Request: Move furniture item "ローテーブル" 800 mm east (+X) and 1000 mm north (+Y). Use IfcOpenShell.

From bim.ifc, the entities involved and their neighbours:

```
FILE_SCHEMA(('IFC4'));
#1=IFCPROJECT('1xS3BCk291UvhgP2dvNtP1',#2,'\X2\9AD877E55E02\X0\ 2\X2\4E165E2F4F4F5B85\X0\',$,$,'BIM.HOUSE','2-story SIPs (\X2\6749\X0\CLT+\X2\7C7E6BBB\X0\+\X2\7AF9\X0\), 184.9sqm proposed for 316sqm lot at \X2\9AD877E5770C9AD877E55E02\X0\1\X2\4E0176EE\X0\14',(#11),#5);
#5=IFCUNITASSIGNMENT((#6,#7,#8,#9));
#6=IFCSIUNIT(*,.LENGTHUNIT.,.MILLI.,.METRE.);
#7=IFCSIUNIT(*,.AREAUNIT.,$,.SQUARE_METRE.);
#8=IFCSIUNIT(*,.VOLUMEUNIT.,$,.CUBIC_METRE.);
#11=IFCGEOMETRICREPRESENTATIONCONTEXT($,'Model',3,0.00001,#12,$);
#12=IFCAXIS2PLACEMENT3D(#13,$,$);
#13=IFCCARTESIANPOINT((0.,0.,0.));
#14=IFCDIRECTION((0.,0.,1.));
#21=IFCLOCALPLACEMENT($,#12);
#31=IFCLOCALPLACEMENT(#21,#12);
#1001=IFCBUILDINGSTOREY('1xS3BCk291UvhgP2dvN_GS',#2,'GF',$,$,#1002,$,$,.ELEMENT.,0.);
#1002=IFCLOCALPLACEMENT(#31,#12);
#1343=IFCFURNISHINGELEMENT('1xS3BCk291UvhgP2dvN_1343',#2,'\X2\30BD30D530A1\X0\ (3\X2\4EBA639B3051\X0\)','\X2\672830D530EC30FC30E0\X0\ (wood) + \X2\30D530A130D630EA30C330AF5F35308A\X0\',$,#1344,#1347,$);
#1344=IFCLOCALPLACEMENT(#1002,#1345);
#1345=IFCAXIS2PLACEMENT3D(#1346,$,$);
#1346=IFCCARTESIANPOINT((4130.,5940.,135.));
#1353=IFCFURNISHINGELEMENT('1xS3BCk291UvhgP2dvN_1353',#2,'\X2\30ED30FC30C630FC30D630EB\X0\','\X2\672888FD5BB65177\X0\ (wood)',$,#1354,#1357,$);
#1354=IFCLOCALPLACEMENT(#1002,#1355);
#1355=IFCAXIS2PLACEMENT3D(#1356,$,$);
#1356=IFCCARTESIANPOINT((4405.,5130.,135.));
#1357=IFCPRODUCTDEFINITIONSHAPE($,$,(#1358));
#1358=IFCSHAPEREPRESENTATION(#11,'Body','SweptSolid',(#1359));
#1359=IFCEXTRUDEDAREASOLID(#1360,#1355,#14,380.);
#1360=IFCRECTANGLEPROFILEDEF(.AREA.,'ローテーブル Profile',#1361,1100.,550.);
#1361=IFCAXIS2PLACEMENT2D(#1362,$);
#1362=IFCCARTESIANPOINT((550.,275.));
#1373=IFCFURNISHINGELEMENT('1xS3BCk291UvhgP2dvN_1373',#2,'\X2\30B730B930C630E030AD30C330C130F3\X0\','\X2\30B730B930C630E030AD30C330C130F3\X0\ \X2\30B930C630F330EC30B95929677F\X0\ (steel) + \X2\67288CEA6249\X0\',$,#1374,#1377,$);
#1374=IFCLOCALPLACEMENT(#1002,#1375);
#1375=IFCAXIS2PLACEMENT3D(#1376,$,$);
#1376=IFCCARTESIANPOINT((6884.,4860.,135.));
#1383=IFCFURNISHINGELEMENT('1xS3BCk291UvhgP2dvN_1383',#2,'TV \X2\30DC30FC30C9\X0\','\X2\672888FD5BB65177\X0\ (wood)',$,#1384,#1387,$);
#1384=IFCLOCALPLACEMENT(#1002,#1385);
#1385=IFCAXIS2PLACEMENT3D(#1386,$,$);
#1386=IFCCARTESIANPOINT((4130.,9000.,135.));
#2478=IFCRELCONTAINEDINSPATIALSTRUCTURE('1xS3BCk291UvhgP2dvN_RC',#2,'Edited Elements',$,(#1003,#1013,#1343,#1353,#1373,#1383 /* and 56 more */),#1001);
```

```python
import ifcopenshell
import ifcopenshell.api.geometry
import ifcopenshell.util.placement
import ifcopenshell.util.unit

model = ifcopenshell.open("bim.ifc")
unit_scale = ifcopenshell.util.unit.calculate_unit_scale(model)

item = model.by_id(1353)
matrix = ifcopenshell.util.placement.get_local_placement(item.ObjectPlacement)
matrix[0, 3] += 0.8 / unit_scale
matrix[1, 3] += 1 / unit_scale
ifcopenshell.api.geometry.edit_object_placement(model, product=item, matrix=matrix, is_si=False)

print(ifcopenshell.util.placement.get_local_placement(item.ObjectPlacement).round(3) + 0.0)

model.write("bim_updated.ifc")
```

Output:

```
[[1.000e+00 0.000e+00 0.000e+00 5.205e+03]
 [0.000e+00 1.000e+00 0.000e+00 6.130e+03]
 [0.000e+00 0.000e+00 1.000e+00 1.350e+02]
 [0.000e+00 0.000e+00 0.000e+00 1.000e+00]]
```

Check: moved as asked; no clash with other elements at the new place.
